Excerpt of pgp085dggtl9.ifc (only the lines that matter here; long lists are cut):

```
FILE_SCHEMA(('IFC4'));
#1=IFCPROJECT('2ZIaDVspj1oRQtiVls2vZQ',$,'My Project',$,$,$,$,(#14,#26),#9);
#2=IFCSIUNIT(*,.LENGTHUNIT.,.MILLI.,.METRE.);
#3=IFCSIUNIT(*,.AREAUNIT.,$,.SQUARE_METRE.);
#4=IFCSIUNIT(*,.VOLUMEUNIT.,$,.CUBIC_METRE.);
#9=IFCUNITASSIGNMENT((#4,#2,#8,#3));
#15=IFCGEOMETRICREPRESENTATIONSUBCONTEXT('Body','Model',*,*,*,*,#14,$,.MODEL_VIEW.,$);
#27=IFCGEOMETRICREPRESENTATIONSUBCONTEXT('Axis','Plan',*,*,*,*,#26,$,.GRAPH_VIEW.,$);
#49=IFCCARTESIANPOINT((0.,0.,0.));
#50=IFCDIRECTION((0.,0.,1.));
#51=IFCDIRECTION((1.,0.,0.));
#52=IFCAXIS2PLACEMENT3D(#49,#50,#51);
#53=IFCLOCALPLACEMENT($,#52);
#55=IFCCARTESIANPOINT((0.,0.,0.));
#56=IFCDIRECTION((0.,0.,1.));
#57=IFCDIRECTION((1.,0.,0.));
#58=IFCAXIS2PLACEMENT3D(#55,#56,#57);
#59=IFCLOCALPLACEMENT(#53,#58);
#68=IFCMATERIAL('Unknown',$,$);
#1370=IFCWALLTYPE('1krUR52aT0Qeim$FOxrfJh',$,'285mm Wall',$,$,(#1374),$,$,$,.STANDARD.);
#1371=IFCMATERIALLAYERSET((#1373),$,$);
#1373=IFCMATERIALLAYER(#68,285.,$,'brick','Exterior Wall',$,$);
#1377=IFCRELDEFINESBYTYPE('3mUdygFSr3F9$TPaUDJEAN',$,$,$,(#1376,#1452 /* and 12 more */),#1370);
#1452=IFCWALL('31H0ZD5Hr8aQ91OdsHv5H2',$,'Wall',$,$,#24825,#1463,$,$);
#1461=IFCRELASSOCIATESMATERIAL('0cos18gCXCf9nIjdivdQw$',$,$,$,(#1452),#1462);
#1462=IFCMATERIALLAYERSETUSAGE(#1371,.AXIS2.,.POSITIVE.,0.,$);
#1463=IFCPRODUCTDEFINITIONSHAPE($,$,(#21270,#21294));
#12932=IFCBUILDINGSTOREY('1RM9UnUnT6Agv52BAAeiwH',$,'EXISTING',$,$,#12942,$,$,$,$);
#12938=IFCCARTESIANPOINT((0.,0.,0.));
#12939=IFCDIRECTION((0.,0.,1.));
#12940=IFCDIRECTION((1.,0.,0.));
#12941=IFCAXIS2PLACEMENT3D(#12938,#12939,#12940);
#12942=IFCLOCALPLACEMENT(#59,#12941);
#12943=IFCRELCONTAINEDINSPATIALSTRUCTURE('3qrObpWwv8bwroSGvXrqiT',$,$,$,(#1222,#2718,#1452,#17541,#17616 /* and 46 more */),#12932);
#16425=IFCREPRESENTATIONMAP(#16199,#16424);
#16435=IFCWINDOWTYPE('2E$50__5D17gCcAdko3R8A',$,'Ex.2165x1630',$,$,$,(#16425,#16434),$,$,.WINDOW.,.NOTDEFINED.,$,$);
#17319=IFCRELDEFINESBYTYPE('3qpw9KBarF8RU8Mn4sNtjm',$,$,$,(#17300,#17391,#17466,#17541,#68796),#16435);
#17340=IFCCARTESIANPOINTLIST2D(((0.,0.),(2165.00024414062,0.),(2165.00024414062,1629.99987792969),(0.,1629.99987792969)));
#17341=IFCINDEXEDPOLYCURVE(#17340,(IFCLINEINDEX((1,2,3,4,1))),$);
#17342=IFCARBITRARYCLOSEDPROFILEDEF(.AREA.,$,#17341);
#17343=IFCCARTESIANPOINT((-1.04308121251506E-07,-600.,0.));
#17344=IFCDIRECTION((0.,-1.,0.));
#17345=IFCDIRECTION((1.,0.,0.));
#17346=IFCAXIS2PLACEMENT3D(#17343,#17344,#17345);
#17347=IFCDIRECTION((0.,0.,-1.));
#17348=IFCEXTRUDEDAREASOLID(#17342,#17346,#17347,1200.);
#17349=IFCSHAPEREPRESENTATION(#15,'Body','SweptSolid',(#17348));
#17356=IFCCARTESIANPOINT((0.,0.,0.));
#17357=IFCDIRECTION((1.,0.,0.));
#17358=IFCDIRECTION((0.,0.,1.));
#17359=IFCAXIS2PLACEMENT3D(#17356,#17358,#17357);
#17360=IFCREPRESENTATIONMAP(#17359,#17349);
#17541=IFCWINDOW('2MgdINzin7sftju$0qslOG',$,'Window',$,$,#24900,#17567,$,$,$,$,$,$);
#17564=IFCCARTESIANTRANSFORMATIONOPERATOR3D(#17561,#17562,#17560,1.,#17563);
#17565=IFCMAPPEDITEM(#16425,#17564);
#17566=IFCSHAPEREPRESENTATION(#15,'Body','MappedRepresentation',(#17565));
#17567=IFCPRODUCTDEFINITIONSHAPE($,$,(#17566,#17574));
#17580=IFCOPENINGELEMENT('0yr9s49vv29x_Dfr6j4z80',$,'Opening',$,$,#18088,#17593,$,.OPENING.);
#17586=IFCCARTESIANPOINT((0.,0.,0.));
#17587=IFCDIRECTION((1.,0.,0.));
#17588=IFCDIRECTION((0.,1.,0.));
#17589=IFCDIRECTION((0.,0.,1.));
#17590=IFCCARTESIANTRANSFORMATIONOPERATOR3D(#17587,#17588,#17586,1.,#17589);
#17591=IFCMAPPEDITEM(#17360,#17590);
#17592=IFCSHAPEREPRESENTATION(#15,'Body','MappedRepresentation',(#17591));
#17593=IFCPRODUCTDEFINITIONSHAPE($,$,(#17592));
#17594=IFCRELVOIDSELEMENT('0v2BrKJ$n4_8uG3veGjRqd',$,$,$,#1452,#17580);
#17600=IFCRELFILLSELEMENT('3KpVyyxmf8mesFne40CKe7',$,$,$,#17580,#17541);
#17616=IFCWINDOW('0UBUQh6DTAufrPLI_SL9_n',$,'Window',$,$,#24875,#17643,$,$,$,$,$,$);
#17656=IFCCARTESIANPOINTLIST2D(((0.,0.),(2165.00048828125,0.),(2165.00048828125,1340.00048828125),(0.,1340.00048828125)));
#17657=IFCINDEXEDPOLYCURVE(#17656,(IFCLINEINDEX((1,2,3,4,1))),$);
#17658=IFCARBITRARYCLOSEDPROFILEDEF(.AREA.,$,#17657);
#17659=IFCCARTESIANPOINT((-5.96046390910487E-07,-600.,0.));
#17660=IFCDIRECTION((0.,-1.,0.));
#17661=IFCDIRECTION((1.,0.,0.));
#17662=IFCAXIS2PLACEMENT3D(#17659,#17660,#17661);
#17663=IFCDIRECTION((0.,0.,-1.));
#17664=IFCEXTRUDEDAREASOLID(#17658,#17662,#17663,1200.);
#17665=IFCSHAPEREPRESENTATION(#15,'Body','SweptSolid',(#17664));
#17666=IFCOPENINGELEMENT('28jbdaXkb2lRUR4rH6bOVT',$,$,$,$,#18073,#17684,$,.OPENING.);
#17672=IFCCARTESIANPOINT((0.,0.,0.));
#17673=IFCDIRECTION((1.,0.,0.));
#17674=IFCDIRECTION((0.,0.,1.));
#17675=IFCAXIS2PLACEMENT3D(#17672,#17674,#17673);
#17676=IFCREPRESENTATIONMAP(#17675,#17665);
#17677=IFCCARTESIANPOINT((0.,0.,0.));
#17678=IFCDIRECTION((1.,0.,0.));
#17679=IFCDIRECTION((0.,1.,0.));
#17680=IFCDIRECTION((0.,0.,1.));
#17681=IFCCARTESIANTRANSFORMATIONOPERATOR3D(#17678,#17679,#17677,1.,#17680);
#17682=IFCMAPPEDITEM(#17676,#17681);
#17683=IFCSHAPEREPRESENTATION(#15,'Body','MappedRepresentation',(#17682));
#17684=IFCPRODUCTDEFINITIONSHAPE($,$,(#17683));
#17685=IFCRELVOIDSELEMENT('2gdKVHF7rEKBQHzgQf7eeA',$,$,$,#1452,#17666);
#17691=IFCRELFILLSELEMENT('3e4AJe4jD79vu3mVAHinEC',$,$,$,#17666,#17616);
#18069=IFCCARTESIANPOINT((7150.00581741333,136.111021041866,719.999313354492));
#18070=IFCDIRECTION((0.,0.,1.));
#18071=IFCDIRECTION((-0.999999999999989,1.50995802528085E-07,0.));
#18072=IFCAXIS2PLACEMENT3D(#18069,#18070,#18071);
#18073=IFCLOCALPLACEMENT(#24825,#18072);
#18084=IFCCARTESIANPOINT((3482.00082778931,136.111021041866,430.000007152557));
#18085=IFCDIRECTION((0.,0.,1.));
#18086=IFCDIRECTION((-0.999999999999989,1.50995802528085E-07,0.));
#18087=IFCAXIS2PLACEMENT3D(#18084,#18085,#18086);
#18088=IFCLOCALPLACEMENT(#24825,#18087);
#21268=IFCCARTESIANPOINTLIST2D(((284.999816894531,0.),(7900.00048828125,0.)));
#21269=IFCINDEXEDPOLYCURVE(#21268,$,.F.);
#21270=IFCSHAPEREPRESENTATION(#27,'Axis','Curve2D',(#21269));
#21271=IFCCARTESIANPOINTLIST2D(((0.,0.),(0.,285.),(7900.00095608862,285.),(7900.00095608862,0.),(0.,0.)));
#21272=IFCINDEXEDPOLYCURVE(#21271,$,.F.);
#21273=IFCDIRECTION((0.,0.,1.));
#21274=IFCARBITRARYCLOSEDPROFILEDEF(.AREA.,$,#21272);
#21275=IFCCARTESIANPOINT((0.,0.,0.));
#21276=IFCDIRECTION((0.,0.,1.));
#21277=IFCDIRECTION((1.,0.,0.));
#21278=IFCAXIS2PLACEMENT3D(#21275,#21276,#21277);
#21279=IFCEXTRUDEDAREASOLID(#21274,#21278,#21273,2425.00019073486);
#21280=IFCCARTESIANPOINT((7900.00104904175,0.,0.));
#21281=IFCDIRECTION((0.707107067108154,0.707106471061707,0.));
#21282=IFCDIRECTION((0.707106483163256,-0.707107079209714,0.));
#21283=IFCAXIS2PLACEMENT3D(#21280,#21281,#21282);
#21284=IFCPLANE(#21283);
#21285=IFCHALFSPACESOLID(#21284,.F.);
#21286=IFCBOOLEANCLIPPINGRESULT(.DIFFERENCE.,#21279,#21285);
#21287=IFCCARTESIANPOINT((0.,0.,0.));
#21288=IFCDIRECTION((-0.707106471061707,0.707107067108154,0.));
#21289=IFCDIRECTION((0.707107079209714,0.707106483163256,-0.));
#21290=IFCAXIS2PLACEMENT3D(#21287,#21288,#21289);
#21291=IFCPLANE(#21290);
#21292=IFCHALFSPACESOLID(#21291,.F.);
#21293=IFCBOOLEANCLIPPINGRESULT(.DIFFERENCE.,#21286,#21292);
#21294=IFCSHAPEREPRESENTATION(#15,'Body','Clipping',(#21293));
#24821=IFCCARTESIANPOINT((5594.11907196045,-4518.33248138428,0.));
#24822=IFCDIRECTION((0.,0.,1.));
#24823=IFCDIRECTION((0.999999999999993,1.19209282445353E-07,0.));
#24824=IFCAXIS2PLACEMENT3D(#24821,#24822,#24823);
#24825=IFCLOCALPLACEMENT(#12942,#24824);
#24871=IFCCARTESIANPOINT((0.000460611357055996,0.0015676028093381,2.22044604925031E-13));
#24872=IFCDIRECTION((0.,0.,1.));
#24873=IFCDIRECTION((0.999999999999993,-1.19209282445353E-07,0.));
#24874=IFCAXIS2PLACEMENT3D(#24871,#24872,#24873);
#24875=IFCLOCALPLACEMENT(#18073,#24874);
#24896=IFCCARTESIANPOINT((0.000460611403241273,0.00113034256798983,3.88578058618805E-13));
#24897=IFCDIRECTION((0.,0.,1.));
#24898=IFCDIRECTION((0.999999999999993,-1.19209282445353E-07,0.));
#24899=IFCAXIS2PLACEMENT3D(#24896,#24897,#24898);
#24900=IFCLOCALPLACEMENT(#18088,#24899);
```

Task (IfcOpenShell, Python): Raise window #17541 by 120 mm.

```python
import numpy as np
import ifcopenshell
import ifcopenshell.api.geometry
import ifcopenshell.util.placement
import ifcopenshell.util.unit

model = ifcopenshell.open("pgp085dggtl9.ifc")
unit_scale = ifcopenshell.util.unit.calculate_unit_scale(model)

window = model.by_guid("2MgdINzin7sftju$0qslOG")
opening = window.FillsVoids[0].RelatingOpeningElement
dz = 120.0

shift = np.array([0.0, 0.0, dz])
# The window is placed relative to its opening, so it follows when the opening moves.
matrix = ifcopenshell.util.placement.get_local_placement(opening.ObjectPlacement)
matrix[:3, 3] += shift
ifcopenshell.api.geometry.edit_object_placement(
    model, product=opening, matrix=matrix, is_si=False, should_transform_children=True
)

print(f"moved by {dz * unit_scale:+.3f} m")

model.write("pgp085dggtl9_updated.ifc")
```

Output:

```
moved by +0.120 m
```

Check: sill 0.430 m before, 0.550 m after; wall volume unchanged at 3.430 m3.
